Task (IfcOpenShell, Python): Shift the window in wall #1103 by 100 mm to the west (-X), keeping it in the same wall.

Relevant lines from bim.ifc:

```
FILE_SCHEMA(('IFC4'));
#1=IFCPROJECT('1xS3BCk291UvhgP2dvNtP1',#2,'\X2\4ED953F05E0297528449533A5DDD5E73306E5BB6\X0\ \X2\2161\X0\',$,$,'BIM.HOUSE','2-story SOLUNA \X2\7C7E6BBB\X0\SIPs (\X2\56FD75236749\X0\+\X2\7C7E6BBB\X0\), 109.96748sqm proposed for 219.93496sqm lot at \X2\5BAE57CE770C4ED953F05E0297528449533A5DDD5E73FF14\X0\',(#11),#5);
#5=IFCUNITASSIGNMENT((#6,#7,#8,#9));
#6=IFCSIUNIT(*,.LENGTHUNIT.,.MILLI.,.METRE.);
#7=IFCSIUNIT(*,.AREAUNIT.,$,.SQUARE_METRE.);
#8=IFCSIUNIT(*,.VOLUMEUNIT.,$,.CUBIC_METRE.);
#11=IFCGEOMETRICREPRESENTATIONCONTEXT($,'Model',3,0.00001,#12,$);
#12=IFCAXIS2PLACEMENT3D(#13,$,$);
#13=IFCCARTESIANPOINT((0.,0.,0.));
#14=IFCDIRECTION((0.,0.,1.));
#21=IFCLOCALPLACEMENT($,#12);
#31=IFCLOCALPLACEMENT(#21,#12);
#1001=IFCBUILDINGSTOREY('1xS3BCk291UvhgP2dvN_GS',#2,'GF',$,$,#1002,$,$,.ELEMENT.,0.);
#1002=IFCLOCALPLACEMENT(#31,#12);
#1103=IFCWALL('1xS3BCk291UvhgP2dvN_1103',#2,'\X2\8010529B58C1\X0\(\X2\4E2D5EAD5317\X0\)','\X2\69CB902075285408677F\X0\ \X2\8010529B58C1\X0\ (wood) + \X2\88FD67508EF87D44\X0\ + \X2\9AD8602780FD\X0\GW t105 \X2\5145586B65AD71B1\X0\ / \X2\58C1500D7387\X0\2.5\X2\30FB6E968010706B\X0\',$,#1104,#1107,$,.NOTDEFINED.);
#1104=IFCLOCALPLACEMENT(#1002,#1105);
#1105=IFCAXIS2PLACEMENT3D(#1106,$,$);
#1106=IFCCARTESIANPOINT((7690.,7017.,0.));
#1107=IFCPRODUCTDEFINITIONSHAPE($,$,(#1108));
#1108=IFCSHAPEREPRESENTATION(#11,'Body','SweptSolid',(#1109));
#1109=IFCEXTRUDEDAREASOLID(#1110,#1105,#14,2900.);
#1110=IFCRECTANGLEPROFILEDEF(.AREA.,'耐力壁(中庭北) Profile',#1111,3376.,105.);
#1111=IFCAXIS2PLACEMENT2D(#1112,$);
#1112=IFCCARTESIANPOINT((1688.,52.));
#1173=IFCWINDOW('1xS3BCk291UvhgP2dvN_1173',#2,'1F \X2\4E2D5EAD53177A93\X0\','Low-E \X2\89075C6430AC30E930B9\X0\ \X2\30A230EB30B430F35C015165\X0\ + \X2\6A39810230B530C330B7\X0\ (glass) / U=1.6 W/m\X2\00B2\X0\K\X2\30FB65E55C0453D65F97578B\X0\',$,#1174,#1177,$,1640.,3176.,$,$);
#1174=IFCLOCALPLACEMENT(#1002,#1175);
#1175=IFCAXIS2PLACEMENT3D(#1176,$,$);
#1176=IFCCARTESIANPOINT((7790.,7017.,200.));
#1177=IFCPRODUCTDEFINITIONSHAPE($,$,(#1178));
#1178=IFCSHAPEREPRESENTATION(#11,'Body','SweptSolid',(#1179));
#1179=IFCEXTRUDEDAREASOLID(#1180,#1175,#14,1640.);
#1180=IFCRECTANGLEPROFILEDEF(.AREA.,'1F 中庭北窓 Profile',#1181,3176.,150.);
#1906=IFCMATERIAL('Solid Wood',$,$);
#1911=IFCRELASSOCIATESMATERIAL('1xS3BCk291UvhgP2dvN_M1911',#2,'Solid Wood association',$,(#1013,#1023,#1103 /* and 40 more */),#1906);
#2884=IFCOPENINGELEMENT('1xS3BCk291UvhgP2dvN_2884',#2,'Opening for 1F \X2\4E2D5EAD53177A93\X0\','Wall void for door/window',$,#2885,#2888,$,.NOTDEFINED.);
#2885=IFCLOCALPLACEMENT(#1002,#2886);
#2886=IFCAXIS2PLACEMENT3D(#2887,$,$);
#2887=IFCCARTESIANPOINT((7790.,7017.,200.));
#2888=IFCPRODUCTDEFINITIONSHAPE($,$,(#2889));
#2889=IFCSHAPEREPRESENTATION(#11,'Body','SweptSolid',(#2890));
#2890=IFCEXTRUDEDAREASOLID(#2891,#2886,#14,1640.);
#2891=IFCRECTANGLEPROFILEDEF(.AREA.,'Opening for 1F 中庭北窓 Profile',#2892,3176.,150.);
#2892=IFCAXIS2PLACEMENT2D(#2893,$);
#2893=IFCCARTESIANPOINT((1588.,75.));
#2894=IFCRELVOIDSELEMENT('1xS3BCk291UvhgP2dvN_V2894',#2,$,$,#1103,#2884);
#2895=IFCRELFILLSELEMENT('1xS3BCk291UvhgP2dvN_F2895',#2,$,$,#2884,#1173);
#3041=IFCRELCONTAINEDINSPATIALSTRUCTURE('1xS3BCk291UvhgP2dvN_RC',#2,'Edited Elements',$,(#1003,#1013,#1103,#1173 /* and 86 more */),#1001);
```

```python
import ifcopenshell
import ifcopenshell.api.geometry
import ifcopenshell.util.placement

model = ifcopenshell.open("bim.ifc")

window = model.by_guid("1xS3BCk291UvhgP2dvN_1173")
opening = window.FillsVoids[0].RelatingOpeningElement
wall = opening.VoidsElements[0].RelatingBuildingElement

wall_matrix = ifcopenshell.util.placement.get_local_placement(wall.ObjectPlacement)
shift = wall_matrix[:3, 0] * -100.0
before = ifcopenshell.util.placement.get_local_placement(window.ObjectPlacement)[:3, 3].copy()

# The window is not placed relative to its opening, so move both.
for product in (opening, window):
    matrix = ifcopenshell.util.placement.get_local_placement(product.ObjectPlacement)
    matrix[:3, 3] += shift
    ifcopenshell.api.geometry.edit_object_placement(model, product=product, matrix=matrix, is_si=False)

after = ifcopenshell.util.placement.get_local_placement(window.ObjectPlacement)[:3, 3]
print("window moved by", (after - before).round(3) + 0.0)

model.write("bim_updated.ifc")
```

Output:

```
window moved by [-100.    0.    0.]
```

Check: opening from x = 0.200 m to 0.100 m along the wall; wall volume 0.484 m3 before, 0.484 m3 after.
